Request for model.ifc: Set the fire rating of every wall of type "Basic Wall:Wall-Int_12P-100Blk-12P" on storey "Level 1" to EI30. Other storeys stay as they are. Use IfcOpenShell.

First a look at what the model holds.

```python
import ifcopenshell
import ifcopenshell.util.element

model = ifcopenshell.open("model.ifc")
print(model.schema)
storey = next(s for s in model.by_type("IfcBuildingStorey") if s.Name == "Level 1")
walls = [e for e in ifcopenshell.util.element.get_decomposition(storey) if e.is_a("IfcWall")]
seen = {}
for e in walls:
    element_type = ifcopenshell.util.element.get_type(e)
    key = (element_type.Name if element_type != e and element_type else None, ifcopenshell.util.element.get_pset(e, "Pset_WallCommon", "FireRating"))
    seen[key] = seen.get(key, 0) + 1
for (name, value), count in sorted(seen.items(), key=str):
    print(count, "x", name, "|", value)
```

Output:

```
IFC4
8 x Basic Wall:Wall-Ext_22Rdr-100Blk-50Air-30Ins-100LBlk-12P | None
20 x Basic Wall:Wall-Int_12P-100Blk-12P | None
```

```python
import ifcopenshell
import ifcopenshell.api.pset
import ifcopenshell.util.element

model = ifcopenshell.open("model.ifc")

storey = next(s for s in model.by_type("IfcBuildingStorey") if s.Name == "Level 1")
walls = [e for e in ifcopenshell.util.element.get_decomposition(storey) if e.is_a("IfcWall")]

count = 0
for e in walls:
    element_type = ifcopenshell.util.element.get_type(e)
    if element_type in (None, e) or element_type.Name != "Basic Wall:Wall-Int_12P-100Blk-12P":
        continue
    # add_pset returns the element's existing set when there is one.
    pset = ifcopenshell.api.pset.add_pset(model, product=e, name="Pset_WallCommon")
    ifcopenshell.api.pset.edit_pset(model, pset=pset, properties={"FireRating": "EI30"})
    count += 1

print(count, "walls updated")

model.write("model_edited.ifc")
```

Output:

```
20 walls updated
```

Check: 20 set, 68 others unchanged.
